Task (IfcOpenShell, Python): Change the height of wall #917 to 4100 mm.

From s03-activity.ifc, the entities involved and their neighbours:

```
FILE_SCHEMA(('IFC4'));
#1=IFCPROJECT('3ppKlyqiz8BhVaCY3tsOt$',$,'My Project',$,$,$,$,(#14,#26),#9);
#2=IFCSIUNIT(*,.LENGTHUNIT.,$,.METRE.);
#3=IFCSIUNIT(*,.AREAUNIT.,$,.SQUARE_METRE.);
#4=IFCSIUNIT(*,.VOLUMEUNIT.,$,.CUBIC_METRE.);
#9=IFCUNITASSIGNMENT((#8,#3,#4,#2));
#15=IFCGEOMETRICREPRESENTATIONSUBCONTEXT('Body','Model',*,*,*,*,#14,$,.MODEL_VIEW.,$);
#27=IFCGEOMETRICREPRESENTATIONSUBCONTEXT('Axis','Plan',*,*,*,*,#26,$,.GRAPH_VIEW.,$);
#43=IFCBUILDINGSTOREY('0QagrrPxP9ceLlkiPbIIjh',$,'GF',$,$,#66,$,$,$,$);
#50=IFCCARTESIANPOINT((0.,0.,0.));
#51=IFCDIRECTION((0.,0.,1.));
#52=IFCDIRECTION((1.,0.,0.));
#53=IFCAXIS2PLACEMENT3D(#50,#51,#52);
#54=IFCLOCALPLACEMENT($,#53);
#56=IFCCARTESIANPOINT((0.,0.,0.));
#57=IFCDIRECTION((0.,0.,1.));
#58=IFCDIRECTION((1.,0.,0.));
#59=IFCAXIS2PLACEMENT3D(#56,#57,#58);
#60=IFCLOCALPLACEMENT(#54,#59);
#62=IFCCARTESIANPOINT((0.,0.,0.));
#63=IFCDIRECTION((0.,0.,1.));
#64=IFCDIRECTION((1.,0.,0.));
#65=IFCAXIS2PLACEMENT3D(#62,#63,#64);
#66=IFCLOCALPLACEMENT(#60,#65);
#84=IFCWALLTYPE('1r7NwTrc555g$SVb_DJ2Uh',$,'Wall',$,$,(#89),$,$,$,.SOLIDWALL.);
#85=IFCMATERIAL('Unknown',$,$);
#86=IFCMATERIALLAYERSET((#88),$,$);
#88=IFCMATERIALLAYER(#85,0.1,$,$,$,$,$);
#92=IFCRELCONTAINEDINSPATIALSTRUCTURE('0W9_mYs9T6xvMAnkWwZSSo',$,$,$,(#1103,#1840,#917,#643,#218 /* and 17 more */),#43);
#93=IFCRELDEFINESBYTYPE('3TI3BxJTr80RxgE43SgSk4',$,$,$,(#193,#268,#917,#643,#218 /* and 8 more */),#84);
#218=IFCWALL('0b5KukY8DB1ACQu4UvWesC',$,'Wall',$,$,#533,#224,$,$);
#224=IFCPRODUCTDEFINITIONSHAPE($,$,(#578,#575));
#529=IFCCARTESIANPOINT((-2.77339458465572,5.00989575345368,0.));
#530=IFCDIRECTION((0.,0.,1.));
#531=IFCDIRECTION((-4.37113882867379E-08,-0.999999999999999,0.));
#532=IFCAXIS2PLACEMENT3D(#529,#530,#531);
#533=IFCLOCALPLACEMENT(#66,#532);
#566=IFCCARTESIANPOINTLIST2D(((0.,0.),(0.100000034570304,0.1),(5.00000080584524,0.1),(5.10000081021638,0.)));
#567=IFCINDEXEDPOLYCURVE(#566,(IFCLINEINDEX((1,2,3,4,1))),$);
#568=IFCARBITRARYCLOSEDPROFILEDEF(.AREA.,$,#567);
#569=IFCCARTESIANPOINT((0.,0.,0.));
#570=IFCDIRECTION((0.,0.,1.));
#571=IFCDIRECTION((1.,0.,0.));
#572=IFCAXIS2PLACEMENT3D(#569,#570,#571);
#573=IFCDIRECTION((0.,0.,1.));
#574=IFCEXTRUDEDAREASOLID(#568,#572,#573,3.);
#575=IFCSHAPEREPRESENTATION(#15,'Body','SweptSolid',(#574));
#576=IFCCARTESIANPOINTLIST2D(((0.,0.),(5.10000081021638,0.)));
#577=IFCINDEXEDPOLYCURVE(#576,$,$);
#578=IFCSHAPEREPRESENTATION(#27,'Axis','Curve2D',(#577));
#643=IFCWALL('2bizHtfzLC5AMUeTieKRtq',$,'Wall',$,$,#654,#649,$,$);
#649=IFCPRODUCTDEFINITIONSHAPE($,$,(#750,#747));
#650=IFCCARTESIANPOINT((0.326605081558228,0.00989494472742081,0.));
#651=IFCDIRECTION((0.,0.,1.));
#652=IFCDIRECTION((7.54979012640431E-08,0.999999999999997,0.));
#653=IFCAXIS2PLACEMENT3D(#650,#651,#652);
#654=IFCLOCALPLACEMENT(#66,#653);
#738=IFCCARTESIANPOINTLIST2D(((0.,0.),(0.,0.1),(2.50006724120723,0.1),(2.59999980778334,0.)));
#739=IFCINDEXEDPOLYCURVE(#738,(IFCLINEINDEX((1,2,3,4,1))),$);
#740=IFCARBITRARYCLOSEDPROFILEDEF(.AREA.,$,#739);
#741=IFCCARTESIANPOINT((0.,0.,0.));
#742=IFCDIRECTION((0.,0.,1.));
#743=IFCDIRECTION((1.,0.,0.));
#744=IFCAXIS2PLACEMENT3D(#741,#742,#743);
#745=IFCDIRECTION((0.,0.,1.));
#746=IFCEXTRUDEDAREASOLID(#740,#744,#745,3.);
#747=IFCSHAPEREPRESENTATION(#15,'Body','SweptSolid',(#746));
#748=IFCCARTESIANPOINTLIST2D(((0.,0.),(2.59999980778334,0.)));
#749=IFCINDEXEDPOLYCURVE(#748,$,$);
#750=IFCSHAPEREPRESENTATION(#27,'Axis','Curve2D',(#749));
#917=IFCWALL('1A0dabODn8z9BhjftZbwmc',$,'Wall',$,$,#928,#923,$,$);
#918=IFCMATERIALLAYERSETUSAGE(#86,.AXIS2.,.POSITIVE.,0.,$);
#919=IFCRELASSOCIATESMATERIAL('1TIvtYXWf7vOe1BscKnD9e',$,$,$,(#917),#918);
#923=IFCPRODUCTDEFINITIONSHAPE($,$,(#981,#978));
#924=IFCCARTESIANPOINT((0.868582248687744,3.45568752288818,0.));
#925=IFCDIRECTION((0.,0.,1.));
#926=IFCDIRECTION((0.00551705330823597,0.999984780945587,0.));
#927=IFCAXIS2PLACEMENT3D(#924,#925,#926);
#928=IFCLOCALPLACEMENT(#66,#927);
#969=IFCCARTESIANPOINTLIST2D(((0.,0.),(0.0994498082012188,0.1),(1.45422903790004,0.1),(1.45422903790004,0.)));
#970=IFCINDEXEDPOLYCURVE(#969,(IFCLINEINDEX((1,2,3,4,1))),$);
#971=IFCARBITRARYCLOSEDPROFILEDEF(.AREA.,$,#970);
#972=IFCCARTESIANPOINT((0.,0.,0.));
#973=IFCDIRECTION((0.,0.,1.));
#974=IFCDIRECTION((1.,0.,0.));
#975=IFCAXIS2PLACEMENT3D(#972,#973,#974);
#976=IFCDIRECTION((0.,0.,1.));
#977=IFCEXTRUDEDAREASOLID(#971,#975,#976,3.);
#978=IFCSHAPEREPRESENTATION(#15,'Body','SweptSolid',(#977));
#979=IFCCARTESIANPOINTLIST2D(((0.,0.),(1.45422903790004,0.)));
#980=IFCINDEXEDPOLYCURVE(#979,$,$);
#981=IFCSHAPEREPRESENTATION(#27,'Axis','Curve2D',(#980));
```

```python
import ifcopenshell
import ifcopenshell.geom
import ifcopenshell.util.representation
import ifcopenshell.util.shape
import ifcopenshell.util.unit

model = ifcopenshell.open("s03-activity.ifc")
unit_scale = ifcopenshell.util.unit.calculate_unit_scale(model)
settings = ifcopenshell.geom.settings()


def volume(element):
    """Net volume in cubic metres, openings subtracted."""
    shape = ifcopenshell.geom.create_shape(settings, element)
    return ifcopenshell.util.shape.get_volume(shape.geometry)


wall = model.by_guid("1A0dabODn8z9BhjftZbwmc")
before = volume(wall)

body = ifcopenshell.util.representation.get_representation(wall, "Model", "Body")
solid = body.Items[0]
old_height = solid.Depth
solid.Depth = 4.1 / unit_scale
after = volume(wall)

print(f"height {old_height:g} -> {solid.Depth:g}, volume {before:.3f} -> {after:.3f} m3")

model.write("s03-activity_updated.ifc")
```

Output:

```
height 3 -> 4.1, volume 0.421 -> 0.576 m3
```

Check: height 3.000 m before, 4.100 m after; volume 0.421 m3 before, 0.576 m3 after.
